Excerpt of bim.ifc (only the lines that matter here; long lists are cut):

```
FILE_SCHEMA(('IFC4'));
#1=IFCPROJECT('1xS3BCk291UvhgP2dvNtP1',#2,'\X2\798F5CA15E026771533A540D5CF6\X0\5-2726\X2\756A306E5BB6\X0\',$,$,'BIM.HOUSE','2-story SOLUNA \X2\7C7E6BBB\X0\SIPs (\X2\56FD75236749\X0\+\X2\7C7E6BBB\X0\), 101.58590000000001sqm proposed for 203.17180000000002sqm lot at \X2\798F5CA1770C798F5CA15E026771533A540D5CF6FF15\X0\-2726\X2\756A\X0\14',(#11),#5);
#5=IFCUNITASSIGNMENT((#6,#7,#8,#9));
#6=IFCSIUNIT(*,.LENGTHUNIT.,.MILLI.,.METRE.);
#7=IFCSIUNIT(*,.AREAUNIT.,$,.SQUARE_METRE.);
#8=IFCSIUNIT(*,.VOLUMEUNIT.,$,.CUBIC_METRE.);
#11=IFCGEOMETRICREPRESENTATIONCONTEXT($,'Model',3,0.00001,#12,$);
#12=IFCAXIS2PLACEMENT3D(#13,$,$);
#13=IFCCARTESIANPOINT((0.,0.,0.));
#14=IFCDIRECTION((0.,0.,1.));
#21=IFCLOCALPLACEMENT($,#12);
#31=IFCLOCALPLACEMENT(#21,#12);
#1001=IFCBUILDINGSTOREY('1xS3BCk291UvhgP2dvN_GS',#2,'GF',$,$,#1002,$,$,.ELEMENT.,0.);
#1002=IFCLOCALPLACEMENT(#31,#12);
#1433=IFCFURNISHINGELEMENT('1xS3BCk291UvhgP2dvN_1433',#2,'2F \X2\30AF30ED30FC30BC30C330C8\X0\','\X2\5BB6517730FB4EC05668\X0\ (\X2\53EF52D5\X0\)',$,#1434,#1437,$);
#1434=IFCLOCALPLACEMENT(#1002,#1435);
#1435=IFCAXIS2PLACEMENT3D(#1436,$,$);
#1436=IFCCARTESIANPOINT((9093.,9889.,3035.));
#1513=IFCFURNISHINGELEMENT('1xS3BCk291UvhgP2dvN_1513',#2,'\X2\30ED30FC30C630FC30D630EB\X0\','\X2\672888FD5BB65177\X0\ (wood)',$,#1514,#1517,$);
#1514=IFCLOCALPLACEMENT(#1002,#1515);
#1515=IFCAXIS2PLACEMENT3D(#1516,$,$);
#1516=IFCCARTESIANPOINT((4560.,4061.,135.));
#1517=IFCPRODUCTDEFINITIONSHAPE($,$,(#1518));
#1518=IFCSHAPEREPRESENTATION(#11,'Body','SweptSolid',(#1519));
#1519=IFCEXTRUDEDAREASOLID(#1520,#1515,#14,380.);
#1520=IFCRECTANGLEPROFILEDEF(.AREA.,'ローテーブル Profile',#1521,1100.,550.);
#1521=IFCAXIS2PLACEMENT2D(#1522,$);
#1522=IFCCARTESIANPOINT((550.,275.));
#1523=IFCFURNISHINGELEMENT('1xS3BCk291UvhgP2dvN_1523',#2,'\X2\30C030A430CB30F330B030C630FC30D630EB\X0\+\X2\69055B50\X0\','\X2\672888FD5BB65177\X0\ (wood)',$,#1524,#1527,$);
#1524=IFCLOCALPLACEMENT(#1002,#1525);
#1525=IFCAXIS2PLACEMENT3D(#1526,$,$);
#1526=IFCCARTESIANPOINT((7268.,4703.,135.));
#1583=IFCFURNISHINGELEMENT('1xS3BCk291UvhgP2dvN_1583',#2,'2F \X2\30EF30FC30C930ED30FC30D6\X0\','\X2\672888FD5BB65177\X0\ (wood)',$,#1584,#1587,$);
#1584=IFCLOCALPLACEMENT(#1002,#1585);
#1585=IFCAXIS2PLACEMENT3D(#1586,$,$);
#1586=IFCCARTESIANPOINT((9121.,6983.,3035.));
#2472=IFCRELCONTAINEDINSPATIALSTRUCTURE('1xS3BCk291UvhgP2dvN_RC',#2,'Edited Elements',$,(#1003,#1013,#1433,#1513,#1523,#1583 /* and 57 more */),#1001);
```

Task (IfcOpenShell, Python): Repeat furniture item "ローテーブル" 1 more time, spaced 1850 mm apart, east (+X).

```python
import numpy as np
import ifcopenshell
import ifcopenshell.api.geometry
import ifcopenshell.api.root
import ifcopenshell.util.element
import ifcopenshell.util.placement
import ifcopenshell.util.unit

model = ifcopenshell.open("bim.ifc")
unit_scale = ifcopenshell.util.unit.calculate_unit_scale(model)


def reuse_history(source, copy):
    """copy_class also copies each property set's owner history, people and application; keep the originals."""
    for rel in copy.IsDefinedBy:
        if rel.is_a("IfcRelDefinesByProperties") and (history := rel.RelatingPropertyDefinition.OwnerHistory):
            rel.RelatingPropertyDefinition.OwnerHistory = source.OwnerHistory
            ifcopenshell.util.element.remove_deep2(model, history)


source = model.by_guid("1xS3BCk291UvhgP2dvN_1513")
base = ifcopenshell.util.placement.get_local_placement(source.ObjectPlacement)
step = np.array([1.0, 0.0, 0.0]) * 1.85 / unit_scale

for i in range(1, 2):
    copy = ifcopenshell.api.root.copy_class(model, product=source)
    copy.Representation = ifcopenshell.util.element.copy_deep(
        model, source.Representation, exclude=["IfcGeometricRepresentationContext", "IfcRepresentationMap"]
    )
    reuse_history(source, copy)
    matrix = base.copy()
    matrix[:3, 3] += i * step
    print("added at", matrix[:3, 3].round(3) + 0.0)
    ifcopenshell.api.geometry.edit_object_placement(model, product=copy, matrix=matrix, is_si=False)

model.write("bim_updated.ifc")
```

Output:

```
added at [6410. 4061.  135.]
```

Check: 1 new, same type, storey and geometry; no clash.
